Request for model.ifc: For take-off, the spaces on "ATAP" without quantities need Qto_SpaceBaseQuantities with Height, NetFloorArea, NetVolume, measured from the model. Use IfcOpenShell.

First a look at what the model holds.

```python
import ifcopenshell
import ifcopenshell.util.element
import ifcopenshell.util.unit

model = ifcopenshell.open("model.ifc")
print(model.schema)
for unit_type in ("LENGTHUNIT", "AREAUNIT", "VOLUMEUNIT"):
    print(unit_type, ifcopenshell.util.unit.calculate_unit_scale(model, unit_type))
storey = next(s for s in model.by_type("IfcBuildingStorey") if s.Name == "ATAP")
spaces = [e for e in ifcopenshell.util.element.get_decomposition(storey) if e.is_a("IfcSpace")]
for e in sorted(spaces, key=lambda e: e.id()):
    print(e.id(), e.is_a(), e.Name, list(ifcopenshell.util.element.get_psets(e, qtos_only=True)), sep=" | ")
```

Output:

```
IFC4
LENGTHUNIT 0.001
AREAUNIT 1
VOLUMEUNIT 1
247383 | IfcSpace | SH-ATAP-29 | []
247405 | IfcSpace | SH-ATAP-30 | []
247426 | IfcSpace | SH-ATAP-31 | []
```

```python
import ifcopenshell
import ifcopenshell.api.pset
import ifcopenshell.geom
import ifcopenshell.util.element
import ifcopenshell.util.shape
import ifcopenshell.util.unit

model = ifcopenshell.open("model.ifc")
unit_scale = ifcopenshell.util.unit.calculate_unit_scale(model)
area_scale = ifcopenshell.util.unit.calculate_unit_scale(model, "AREAUNIT")
volume_scale = ifcopenshell.util.unit.calculate_unit_scale(model, "VOLUMEUNIT")
settings = ifcopenshell.geom.settings()

storey = next(s for s in model.by_type("IfcBuildingStorey") if s.Name == "ATAP")
spaces = [e for e in ifcopenshell.util.element.get_decomposition(storey) if e.is_a("IfcSpace")]

for e in sorted(spaces, key=lambda e: e.id()):
    if ifcopenshell.util.element.get_psets(e, qtos_only=True, should_inherit=False):
        continue
    # Geometry comes back in metres, in the element's own axes.
    shape = ifcopenshell.geom.create_shape(settings, e)
    values = {
        "Height": ifcopenshell.util.shape.get_z(shape.geometry) / unit_scale,
        "NetFloorArea": ifcopenshell.util.shape.get_footprint_area(shape.geometry) / area_scale,
        "NetVolume": ifcopenshell.util.shape.get_volume(shape.geometry) / volume_scale,
    }
    qto = ifcopenshell.api.pset.add_qto(model, product=e, name="Qto_SpaceBaseQuantities")
    ifcopenshell.api.pset.edit_qto(model, qto=qto, properties=values)
    print(e.id(), {k: round(v, 3) for k, v in values.items()})

model.write("model_rev.ifc")
```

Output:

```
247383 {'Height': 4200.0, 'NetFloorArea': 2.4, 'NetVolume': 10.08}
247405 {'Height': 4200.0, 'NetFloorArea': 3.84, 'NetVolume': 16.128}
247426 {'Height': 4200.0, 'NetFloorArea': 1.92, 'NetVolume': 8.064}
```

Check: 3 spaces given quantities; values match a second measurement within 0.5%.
